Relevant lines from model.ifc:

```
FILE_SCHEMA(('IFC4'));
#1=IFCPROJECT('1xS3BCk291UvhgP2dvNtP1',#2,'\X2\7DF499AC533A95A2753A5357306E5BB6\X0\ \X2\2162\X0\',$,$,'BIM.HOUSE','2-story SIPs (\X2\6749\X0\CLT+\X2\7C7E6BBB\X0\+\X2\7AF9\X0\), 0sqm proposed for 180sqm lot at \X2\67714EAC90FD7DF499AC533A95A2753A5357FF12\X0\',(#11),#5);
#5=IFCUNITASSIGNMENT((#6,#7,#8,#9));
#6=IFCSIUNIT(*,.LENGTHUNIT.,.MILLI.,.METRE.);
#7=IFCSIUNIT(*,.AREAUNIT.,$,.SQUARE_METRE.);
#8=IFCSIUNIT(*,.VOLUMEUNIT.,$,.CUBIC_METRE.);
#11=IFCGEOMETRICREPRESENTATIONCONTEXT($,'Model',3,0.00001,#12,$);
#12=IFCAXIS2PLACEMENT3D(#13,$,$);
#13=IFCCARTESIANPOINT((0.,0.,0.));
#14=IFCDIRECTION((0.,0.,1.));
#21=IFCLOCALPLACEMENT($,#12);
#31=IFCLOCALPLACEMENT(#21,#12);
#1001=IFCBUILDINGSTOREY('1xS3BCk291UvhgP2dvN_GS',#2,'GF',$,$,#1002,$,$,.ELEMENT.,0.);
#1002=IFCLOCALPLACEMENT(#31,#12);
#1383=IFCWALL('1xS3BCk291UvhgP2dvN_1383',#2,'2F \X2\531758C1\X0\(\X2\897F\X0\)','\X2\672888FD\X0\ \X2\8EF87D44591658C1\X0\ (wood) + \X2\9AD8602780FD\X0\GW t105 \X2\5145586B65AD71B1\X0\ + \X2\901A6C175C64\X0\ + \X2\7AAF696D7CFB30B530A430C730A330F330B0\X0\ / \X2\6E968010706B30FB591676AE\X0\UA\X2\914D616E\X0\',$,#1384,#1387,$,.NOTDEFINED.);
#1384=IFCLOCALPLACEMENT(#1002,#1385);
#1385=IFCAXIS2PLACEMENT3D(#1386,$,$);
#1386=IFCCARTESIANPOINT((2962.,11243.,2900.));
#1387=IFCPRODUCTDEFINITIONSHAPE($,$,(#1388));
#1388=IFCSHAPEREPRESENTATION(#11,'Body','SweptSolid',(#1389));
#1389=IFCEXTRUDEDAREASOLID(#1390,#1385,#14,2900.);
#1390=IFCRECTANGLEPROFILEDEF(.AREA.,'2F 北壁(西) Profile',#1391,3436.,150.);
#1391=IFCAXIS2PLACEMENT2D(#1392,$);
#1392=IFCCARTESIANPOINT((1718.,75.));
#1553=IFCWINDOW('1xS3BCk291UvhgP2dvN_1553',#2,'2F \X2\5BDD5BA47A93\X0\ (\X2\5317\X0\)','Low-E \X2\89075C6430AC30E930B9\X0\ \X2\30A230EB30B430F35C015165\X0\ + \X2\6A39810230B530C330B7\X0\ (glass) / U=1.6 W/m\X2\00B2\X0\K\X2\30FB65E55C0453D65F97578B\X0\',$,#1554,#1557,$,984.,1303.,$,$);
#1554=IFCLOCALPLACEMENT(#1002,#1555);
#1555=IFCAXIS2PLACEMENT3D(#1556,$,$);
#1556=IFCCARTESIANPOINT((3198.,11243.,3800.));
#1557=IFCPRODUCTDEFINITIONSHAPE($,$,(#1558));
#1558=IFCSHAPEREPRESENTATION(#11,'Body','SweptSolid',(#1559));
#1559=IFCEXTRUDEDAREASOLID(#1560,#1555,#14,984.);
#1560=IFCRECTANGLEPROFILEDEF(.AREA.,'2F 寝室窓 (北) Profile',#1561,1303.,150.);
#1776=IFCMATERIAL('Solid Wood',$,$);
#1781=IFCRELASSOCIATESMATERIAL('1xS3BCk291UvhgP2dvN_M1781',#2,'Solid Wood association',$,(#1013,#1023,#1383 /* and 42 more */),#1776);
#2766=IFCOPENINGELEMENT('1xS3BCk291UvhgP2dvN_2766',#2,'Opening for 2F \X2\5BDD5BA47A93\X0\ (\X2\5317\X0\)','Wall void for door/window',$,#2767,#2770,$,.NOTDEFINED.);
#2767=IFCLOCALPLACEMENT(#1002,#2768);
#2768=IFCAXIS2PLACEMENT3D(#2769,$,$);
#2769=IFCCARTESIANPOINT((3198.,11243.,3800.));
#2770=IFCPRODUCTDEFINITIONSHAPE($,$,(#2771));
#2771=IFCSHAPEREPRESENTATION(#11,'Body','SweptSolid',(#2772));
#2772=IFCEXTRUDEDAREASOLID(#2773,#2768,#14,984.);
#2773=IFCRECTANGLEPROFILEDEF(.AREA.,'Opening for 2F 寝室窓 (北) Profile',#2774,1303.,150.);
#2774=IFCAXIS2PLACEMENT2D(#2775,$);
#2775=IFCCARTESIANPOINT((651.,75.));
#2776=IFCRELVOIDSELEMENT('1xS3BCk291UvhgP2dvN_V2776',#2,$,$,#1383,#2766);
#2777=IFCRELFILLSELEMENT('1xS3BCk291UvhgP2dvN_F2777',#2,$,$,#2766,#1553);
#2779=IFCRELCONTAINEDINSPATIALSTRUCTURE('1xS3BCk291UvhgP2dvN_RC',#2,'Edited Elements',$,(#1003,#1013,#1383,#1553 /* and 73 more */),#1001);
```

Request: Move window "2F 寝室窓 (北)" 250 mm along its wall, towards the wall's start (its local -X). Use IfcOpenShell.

```python
import ifcopenshell
import ifcopenshell.api.geometry
import ifcopenshell.util.placement
import ifcopenshell.util.unit

model = ifcopenshell.open("model.ifc")
unit_scale = ifcopenshell.util.unit.calculate_unit_scale(model)

window = model.by_guid("1xS3BCk291UvhgP2dvN_1553")
opening = window.FillsVoids[0].RelatingOpeningElement
wall = opening.VoidsElements[0].RelatingBuildingElement

wall_matrix = ifcopenshell.util.placement.get_local_placement(wall.ObjectPlacement)
shift = wall_matrix[:3, 0] * -0.25 / unit_scale
before = ifcopenshell.util.placement.get_local_placement(window.ObjectPlacement)[:3, 3].copy()

# The window is not placed relative to its opening, so move both.
for product in (opening, window):
    matrix = ifcopenshell.util.placement.get_local_placement(product.ObjectPlacement)
    matrix[:3, 3] += shift
    ifcopenshell.api.geometry.edit_object_placement(model, product=product, matrix=matrix, is_si=False)

after = ifcopenshell.util.placement.get_local_placement(window.ObjectPlacement)[:3, 3]
print("window moved by", (after - before).round(3) + 0.0)

model.write("model_v2.ifc")
```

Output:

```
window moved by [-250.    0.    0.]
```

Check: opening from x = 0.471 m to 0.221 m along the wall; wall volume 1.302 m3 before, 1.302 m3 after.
